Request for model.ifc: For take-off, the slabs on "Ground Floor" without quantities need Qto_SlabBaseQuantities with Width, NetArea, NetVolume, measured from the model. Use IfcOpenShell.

First a look at what the model holds.

```python
import ifcopenshell
import ifcopenshell.util.element
import ifcopenshell.util.unit

model = ifcopenshell.open("model.ifc")
print(model.schema)
for unit_type in ("LENGTHUNIT", "AREAUNIT", "VOLUMEUNIT"):
    print(unit_type, ifcopenshell.util.unit.calculate_unit_scale(model, unit_type))
storey = next(s for s in model.by_type("IfcBuildingStorey") if s.Name == "Ground Floor")
slabs = [e for e in ifcopenshell.util.element.get_decomposition(storey) if e.is_a("IfcSlab")]
for e in sorted(slabs, key=lambda e: e.id()):
    print(e.id(), e.is_a(), e.Name, list(ifcopenshell.util.element.get_psets(e, qtos_only=True)), sep=" | ")
```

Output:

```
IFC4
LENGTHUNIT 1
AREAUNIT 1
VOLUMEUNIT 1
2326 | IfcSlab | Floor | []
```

```python
import ifcopenshell
import ifcopenshell.api.pset
import ifcopenshell.geom
import ifcopenshell.util.element
import ifcopenshell.util.shape
import ifcopenshell.util.unit

model = ifcopenshell.open("model.ifc")
unit_scale = ifcopenshell.util.unit.calculate_unit_scale(model)
area_scale = ifcopenshell.util.unit.calculate_unit_scale(model, "AREAUNIT")
volume_scale = ifcopenshell.util.unit.calculate_unit_scale(model, "VOLUMEUNIT")
settings = ifcopenshell.geom.settings()

storey = next(s for s in model.by_type("IfcBuildingStorey") if s.Name == "Ground Floor")
slabs = [e for e in ifcopenshell.util.element.get_decomposition(storey) if e.is_a("IfcSlab")]

for e in sorted(slabs, key=lambda e: e.id()):
    if ifcopenshell.util.element.get_psets(e, qtos_only=True, should_inherit=False):
        continue
    # Geometry comes back in metres, in the element's own axes.
    shape = ifcopenshell.geom.create_shape(settings, e)
    values = {
        "Width": ifcopenshell.util.shape.get_z(shape.geometry) / unit_scale,
        "NetArea": ifcopenshell.util.shape.get_footprint_area(shape.geometry) / area_scale,
        "NetVolume": ifcopenshell.util.shape.get_volume(shape.geometry) / volume_scale,
    }
    qto = ifcopenshell.api.pset.add_qto(model, product=e, name="Qto_SlabBaseQuantities")
    ifcopenshell.api.pset.edit_qto(model, qto=qto, properties=values)
    print(e.id(), {k: round(v, 3) for k, v in values.items()})

model.write("model_v2.ifc")
```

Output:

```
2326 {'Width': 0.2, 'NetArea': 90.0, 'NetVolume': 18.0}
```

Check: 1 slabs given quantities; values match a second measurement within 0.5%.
